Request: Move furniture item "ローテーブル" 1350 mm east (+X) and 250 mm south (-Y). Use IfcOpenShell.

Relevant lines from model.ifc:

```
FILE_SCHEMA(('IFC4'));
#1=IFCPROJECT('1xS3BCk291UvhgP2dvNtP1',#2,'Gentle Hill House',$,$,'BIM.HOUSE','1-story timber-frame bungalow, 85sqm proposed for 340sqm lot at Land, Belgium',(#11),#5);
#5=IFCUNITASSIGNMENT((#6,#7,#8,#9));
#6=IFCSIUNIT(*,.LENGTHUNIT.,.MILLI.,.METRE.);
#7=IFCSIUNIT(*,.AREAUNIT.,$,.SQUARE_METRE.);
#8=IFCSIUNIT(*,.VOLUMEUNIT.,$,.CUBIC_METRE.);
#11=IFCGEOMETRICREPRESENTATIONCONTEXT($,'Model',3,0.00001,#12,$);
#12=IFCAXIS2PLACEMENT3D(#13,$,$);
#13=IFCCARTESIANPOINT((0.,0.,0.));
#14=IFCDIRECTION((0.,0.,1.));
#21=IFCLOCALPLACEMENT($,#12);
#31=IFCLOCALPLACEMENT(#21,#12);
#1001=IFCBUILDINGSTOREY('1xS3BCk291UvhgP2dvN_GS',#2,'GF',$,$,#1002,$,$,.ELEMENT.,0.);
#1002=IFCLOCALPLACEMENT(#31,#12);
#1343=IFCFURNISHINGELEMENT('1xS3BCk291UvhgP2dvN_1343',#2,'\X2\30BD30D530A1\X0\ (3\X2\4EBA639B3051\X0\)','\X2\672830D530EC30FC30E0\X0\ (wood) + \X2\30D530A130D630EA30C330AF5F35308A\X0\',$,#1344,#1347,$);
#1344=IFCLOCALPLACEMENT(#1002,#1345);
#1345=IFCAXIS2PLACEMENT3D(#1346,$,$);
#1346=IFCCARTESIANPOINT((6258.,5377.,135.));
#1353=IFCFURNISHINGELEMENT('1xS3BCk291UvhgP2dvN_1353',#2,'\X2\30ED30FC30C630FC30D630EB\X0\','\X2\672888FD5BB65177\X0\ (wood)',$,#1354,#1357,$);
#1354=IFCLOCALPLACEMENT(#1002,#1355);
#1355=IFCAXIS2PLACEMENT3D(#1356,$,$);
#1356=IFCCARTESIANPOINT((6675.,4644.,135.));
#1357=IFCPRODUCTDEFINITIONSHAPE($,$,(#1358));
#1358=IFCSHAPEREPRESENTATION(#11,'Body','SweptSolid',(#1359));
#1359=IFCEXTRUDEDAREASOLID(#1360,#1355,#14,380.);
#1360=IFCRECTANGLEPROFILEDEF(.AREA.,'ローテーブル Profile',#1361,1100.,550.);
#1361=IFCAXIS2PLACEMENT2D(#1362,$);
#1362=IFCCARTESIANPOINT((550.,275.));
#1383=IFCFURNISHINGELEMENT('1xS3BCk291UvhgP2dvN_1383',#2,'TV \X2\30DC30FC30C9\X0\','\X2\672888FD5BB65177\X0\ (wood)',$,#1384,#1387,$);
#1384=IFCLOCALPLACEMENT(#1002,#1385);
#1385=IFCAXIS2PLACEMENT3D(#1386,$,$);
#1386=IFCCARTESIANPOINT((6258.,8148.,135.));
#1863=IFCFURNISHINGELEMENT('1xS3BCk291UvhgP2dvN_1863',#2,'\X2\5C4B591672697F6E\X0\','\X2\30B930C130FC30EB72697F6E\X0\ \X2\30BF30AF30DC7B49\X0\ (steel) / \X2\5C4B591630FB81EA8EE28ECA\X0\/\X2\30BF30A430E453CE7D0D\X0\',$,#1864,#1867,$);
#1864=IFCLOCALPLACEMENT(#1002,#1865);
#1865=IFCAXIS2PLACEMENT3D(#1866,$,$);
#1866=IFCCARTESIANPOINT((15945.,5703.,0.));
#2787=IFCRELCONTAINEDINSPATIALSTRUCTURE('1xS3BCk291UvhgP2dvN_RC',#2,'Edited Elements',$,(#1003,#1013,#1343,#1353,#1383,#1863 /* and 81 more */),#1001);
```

```python
import ifcopenshell
import ifcopenshell.api.geometry
import ifcopenshell.util.placement
import ifcopenshell.util.unit

model = ifcopenshell.open("model.ifc")
unit_scale = ifcopenshell.util.unit.calculate_unit_scale(model)

item = model.by_guid("1xS3BCk291UvhgP2dvN_1353")
matrix = ifcopenshell.util.placement.get_local_placement(item.ObjectPlacement)
matrix[0, 3] += 1.35 / unit_scale
matrix[1, 3] -= 0.25 / unit_scale
ifcopenshell.api.geometry.edit_object_placement(model, product=item, matrix=matrix, is_si=False)

print(ifcopenshell.util.placement.get_local_placement(item.ObjectPlacement).round(3) + 0.0)

model.write("model_edited.ifc")
```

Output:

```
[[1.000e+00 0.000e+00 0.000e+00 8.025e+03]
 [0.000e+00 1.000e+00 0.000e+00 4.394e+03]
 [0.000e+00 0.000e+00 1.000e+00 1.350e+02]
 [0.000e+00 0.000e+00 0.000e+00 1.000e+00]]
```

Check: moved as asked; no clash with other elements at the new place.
